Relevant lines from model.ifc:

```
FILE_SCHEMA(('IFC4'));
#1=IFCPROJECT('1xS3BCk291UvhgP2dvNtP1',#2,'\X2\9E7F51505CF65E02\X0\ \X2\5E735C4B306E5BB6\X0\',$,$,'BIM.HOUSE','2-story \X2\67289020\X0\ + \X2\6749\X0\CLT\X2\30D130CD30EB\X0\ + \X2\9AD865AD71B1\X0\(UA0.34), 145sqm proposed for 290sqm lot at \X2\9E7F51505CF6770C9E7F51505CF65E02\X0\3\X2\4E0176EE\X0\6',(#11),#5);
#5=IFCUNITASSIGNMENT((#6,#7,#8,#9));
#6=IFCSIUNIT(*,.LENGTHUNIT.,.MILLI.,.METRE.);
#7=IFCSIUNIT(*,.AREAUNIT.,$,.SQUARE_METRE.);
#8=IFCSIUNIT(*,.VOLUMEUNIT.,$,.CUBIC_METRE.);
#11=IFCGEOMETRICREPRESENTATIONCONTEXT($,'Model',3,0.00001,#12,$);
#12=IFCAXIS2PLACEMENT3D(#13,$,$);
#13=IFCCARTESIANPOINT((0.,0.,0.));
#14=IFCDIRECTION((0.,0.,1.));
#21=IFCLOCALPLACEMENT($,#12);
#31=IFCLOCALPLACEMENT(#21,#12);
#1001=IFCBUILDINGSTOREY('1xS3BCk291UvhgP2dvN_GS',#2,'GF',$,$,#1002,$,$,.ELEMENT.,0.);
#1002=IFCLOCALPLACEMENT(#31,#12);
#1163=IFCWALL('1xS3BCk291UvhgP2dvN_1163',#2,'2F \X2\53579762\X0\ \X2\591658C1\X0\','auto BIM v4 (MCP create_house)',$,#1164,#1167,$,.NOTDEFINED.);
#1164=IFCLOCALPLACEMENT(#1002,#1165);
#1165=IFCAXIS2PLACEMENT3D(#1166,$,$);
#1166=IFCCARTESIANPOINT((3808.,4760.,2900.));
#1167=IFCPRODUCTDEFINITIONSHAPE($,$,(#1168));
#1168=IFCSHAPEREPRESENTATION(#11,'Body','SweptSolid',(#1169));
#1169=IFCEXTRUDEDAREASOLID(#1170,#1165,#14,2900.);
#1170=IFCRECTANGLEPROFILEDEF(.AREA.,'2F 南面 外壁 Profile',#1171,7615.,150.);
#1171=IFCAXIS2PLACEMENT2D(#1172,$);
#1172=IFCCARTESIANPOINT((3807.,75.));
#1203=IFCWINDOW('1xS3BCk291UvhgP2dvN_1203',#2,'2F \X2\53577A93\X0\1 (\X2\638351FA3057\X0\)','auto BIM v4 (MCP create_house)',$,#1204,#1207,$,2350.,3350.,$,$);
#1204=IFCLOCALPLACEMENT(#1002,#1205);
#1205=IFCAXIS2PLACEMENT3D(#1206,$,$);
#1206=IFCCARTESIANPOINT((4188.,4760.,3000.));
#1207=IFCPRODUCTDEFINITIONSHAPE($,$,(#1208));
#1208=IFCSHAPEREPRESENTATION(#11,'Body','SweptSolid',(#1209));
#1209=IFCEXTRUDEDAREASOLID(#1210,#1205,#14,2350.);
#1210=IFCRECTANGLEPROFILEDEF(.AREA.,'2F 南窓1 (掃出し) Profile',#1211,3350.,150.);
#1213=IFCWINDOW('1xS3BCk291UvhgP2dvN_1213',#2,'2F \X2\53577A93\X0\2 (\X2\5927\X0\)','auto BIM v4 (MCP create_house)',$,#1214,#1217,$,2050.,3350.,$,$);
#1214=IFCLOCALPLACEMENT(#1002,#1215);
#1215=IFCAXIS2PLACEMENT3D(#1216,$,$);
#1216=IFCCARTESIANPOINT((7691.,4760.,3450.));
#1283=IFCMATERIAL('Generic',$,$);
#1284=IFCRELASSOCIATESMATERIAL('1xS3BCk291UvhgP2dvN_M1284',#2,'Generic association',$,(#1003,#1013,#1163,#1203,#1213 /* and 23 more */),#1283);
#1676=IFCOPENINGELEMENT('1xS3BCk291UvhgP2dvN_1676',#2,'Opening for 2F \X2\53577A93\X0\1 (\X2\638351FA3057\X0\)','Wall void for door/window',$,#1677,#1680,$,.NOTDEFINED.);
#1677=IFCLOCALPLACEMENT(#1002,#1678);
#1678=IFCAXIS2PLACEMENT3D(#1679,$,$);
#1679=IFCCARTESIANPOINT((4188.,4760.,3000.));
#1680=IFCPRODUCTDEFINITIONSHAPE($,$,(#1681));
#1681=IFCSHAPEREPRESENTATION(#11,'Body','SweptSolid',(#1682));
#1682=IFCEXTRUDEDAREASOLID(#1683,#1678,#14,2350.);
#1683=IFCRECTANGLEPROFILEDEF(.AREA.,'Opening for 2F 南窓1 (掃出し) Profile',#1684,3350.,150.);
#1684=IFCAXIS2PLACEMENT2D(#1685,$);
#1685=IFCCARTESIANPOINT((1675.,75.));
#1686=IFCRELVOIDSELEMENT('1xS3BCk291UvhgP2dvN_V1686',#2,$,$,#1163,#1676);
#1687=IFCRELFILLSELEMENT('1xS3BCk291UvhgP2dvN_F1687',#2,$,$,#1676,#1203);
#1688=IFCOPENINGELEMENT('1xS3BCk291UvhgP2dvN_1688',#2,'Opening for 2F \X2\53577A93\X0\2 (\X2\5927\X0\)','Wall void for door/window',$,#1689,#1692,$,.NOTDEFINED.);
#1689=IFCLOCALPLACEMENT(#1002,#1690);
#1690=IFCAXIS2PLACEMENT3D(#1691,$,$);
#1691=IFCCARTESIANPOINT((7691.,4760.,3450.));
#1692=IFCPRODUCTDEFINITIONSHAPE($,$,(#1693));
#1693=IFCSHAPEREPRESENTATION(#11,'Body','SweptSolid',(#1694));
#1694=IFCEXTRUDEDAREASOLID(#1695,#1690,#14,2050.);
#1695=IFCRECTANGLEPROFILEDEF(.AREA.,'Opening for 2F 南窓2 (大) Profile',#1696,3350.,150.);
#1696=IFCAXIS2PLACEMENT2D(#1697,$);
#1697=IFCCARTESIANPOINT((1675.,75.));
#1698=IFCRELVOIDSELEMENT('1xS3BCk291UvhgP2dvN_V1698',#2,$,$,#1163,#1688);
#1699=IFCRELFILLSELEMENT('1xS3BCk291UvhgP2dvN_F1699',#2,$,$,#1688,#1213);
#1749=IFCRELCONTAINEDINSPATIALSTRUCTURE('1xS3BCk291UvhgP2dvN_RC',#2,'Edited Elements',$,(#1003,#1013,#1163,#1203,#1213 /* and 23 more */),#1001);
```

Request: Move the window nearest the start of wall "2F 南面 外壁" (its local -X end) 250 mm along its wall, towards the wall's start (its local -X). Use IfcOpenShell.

```python
import ifcopenshell
import ifcopenshell.api.geometry
import ifcopenshell.util.placement
import ifcopenshell.util.unit

model = ifcopenshell.open("model.ifc")
unit_scale = ifcopenshell.util.unit.calculate_unit_scale(model)

window = model.by_guid("1xS3BCk291UvhgP2dvN_1203")
opening = window.FillsVoids[0].RelatingOpeningElement
wall = opening.VoidsElements[0].RelatingBuildingElement

wall_matrix = ifcopenshell.util.placement.get_local_placement(wall.ObjectPlacement)
shift = wall_matrix[:3, 0] * -0.25 / unit_scale
before = ifcopenshell.util.placement.get_local_placement(window.ObjectPlacement)[:3, 3].copy()

# The window is not placed relative to its opening, so move both.
for product in (opening, window):
    matrix = ifcopenshell.util.placement.get_local_placement(product.ObjectPlacement)
    matrix[:3, 3] += shift
    ifcopenshell.api.geometry.edit_object_placement(model, product=product, matrix=matrix, is_si=False)

after = ifcopenshell.util.placement.get_local_placement(window.ObjectPlacement)[:3, 3]
print("window moved by", (after - before).round(3) + 0.0)

model.write("model-out.ifc")
```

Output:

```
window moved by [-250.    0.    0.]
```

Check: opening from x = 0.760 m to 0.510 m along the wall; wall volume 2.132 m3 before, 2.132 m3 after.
